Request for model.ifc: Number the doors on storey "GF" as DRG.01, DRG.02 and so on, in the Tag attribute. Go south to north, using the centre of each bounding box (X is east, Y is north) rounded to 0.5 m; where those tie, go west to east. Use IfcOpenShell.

First a look at what the model holds.

```python
import ifcopenshell
import ifcopenshell.util.element
import ifcopenshell.util.placement

model = ifcopenshell.open("model.ifc")
print(model.schema)
storey = next(s for s in model.by_type("IfcBuildingStorey") if s.Name == "GF")
doors = [e for e in ifcopenshell.util.element.get_decomposition(storey) if e.is_a("IfcDoor")]
for e in sorted(doors, key=lambda e: e.id()):
    origin = ifcopenshell.util.placement.get_local_placement(e.ObjectPlacement)[:3, 3]
    print(e.id(), e.Tag, e.Name, origin.round(2) + 0.0, sep=" | ")
```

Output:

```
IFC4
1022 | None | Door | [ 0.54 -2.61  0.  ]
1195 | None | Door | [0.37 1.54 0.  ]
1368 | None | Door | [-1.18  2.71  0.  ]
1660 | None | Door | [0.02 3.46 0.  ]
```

```python
import ifcopenshell
import ifcopenshell.geom
import ifcopenshell.util.element
import ifcopenshell.util.shape

model = ifcopenshell.open("model.ifc")
settings = ifcopenshell.geom.settings()
settings.set("use-world-coords", True)


def centre(element):
    shape = ifcopenshell.geom.create_shape(settings, element)
    return ifcopenshell.util.shape.get_bbox_centroid(shape.geometry)


storey = next(s for s in model.by_type("IfcBuildingStorey") if s.Name == "GF")
doors = [e for e in ifcopenshell.util.element.get_decomposition(storey) if e.is_a("IfcDoor")]

# Insertion points can sit at a corner or the storey origin, so sort by the geometry (in metres).
centres = {e: centre(e) for e in doors}
doors.sort(key=lambda e: (round(centres[e][1] / 0.5), centres[e][0]))

for i, e in enumerate(doors, start=1):
    number = f"DRG.{i:02d}"
    e.Tag = number
    print(e.id(), number)

model.write("model-out.ifc")
```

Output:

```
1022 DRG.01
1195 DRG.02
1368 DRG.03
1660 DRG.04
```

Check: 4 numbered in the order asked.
